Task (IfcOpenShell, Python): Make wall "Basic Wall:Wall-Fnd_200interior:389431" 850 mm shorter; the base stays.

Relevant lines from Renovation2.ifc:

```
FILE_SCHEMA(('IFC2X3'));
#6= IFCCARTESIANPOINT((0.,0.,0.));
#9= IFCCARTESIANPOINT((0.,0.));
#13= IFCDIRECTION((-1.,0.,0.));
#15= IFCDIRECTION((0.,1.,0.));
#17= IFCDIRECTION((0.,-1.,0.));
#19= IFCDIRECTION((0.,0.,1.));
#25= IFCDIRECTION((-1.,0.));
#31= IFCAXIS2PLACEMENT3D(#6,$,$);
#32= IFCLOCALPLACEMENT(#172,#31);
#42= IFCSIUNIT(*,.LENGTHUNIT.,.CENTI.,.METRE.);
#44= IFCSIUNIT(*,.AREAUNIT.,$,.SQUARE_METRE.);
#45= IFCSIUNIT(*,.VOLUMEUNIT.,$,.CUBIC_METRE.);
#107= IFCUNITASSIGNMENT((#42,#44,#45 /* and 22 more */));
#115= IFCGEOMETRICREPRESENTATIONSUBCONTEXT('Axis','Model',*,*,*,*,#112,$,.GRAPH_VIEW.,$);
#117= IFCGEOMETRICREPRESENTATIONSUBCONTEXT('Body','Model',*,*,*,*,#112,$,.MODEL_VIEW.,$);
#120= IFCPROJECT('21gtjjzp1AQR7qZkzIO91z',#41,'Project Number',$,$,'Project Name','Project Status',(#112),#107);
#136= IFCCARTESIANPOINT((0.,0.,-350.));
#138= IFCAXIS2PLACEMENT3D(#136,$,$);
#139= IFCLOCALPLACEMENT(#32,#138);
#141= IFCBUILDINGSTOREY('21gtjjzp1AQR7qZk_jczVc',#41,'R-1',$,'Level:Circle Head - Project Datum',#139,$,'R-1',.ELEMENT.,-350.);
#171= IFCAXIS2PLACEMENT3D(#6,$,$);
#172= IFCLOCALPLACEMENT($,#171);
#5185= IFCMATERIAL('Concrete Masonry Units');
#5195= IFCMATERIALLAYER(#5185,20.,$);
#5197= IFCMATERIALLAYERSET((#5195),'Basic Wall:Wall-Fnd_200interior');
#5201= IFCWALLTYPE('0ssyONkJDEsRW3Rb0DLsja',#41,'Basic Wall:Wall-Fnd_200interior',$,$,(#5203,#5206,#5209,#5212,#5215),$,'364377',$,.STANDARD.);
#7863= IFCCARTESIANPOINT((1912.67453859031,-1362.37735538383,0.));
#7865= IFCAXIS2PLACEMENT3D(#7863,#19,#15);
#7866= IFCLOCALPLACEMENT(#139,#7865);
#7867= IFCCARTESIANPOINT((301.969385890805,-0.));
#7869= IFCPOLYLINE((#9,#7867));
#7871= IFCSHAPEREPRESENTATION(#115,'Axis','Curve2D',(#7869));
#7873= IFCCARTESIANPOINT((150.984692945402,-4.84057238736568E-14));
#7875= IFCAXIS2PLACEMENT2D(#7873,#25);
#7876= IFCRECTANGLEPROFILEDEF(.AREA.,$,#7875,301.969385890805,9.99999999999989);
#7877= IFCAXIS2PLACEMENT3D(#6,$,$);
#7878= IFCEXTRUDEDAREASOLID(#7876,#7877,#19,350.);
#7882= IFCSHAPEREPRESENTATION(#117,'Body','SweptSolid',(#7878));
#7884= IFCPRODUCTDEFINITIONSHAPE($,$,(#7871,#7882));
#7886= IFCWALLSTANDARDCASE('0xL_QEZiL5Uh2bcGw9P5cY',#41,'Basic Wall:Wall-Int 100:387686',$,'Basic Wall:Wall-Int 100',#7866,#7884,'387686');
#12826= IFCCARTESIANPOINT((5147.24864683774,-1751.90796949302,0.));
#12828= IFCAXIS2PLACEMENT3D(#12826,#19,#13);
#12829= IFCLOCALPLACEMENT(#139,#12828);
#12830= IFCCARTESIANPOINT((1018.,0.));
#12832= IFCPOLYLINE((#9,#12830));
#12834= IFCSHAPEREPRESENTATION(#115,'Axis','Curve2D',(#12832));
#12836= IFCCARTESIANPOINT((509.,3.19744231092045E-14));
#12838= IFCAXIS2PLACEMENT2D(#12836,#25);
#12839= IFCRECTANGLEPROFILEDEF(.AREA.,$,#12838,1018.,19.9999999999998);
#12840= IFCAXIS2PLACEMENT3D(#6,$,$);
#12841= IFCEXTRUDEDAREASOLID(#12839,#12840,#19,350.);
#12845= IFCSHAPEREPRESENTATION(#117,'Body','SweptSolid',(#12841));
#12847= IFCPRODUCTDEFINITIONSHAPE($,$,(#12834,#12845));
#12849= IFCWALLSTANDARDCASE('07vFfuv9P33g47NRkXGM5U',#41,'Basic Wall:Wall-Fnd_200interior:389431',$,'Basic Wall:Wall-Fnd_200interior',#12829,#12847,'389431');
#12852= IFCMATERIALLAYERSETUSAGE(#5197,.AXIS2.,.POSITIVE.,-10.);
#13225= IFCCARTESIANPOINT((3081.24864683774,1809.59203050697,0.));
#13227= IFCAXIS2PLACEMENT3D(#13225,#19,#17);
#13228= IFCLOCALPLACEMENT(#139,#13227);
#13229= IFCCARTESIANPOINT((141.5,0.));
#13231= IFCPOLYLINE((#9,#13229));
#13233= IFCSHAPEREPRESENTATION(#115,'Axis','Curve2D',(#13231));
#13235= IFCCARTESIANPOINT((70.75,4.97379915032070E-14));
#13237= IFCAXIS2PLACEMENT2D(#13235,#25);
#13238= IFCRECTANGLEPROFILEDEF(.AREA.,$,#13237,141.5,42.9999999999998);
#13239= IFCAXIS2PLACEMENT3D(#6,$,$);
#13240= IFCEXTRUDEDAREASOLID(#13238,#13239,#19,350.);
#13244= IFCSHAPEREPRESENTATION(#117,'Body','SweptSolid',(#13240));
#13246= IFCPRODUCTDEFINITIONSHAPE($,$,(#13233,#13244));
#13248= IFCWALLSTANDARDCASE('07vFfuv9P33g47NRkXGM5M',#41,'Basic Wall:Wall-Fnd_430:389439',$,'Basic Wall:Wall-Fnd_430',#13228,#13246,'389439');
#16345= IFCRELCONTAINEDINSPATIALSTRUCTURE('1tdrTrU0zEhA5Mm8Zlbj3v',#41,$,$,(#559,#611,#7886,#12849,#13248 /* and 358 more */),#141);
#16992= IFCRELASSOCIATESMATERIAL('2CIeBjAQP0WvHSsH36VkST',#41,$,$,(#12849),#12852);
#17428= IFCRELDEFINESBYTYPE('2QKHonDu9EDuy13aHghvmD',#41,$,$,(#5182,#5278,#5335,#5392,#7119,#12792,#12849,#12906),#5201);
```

```python
import ifcopenshell
import ifcopenshell.geom
import ifcopenshell.util.representation
import ifcopenshell.util.shape
import ifcopenshell.util.unit

model = ifcopenshell.open("Renovation2.ifc")
unit_scale = ifcopenshell.util.unit.calculate_unit_scale(model)
settings = ifcopenshell.geom.settings()


def volume(element):
    """Net volume in cubic metres, openings subtracted."""
    shape = ifcopenshell.geom.create_shape(settings, element)
    return ifcopenshell.util.shape.get_volume(shape.geometry)


wall = model.by_guid("07vFfuv9P33g47NRkXGM5U")
before = volume(wall)

body = ifcopenshell.util.representation.get_representation(wall, "Model", "Body")
solid = body.Items[0]
old_height = solid.Depth
solid.Depth -= 0.85 / unit_scale
after = volume(wall)

print(f"height {old_height:g} -> {solid.Depth:g}, volume {before:.3f} -> {after:.3f} m3")

model.write("Renovation2_updated.ifc")
```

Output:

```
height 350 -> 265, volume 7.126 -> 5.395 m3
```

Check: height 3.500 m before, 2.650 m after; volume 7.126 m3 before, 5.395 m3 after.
